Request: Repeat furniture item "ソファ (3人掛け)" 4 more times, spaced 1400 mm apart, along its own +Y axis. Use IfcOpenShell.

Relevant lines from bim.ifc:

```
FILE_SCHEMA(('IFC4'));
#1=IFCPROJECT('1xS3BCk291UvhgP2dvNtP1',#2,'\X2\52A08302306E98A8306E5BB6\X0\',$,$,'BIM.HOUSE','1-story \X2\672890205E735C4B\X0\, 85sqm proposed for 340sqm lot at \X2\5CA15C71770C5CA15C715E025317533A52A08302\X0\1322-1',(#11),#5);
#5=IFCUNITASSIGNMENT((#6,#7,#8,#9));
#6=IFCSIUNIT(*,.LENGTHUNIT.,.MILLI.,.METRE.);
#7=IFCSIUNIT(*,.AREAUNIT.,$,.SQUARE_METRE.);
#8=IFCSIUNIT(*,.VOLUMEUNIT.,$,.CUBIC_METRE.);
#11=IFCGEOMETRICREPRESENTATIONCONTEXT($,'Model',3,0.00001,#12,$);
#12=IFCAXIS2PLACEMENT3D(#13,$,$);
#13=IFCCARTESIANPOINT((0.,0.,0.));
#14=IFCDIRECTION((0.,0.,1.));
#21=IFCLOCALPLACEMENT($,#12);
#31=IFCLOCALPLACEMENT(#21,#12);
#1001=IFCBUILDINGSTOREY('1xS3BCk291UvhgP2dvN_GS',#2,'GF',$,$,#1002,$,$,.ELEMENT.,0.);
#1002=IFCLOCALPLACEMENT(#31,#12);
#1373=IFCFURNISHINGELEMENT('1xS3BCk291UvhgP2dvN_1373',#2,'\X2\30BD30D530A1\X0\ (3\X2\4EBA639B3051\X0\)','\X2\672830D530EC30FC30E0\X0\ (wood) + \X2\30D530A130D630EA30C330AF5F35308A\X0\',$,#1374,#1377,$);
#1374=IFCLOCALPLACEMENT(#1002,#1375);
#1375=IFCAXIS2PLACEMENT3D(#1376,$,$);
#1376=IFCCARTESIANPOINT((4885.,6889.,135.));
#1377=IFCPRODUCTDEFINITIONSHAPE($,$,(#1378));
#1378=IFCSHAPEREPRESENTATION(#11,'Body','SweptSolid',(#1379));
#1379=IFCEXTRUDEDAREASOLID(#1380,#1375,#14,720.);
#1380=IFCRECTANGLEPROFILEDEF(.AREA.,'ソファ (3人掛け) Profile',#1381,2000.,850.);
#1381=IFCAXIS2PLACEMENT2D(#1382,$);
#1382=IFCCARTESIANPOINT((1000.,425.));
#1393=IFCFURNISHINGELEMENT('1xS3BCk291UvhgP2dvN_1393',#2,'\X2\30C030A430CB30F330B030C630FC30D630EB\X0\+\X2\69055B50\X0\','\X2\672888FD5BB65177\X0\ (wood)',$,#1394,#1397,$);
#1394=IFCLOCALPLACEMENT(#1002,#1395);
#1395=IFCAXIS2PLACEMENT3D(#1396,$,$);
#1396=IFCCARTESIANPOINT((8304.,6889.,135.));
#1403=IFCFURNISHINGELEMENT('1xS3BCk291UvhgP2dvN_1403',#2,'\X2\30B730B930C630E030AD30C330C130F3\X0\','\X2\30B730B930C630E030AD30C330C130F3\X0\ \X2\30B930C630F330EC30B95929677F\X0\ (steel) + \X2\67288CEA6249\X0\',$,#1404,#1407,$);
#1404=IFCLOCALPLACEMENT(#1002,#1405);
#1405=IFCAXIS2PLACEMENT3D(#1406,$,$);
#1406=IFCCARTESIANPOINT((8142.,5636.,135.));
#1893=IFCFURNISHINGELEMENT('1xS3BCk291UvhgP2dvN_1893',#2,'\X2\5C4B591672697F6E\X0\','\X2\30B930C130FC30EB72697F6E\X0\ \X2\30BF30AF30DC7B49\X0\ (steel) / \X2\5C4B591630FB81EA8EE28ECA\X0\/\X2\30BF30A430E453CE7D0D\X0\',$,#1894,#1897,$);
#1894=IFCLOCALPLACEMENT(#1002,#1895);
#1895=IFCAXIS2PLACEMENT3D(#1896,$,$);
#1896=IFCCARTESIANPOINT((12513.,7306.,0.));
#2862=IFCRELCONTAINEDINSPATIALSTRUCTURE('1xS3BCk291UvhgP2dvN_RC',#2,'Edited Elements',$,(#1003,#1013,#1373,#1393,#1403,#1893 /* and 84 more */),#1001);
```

```python
import ifcopenshell
import ifcopenshell.api.geometry
import ifcopenshell.api.root
import ifcopenshell.util.element
import ifcopenshell.util.placement

model = ifcopenshell.open("bim.ifc")


def reuse_history(source, copy):
    """copy_class also copies each property set's owner history, people and application; keep the originals."""
    for rel in copy.IsDefinedBy:
        if rel.is_a("IfcRelDefinesByProperties") and (history := rel.RelatingPropertyDefinition.OwnerHistory):
            rel.RelatingPropertyDefinition.OwnerHistory = source.OwnerHistory
            ifcopenshell.util.element.remove_deep2(model, history)


source = model.by_id(1373)
base = ifcopenshell.util.placement.get_local_placement(source.ObjectPlacement)
step = base[:3, 1] * 1400.0

for i in range(1, 5):
    copy = ifcopenshell.api.root.copy_class(model, product=source)
    copy.Representation = ifcopenshell.util.element.copy_deep(
        model, source.Representation, exclude=["IfcGeometricRepresentationContext", "IfcRepresentationMap"]
    )
    reuse_history(source, copy)
    matrix = base.copy()
    matrix[:3, 3] += i * step
    print("added at", matrix[:3, 3].round(3) + 0.0)
    ifcopenshell.api.geometry.edit_object_placement(model, product=copy, matrix=matrix, is_si=False)

model.write("bim_v2.ifc")
```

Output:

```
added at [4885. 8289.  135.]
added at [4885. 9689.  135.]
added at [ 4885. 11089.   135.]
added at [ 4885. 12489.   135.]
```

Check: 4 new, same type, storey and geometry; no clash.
